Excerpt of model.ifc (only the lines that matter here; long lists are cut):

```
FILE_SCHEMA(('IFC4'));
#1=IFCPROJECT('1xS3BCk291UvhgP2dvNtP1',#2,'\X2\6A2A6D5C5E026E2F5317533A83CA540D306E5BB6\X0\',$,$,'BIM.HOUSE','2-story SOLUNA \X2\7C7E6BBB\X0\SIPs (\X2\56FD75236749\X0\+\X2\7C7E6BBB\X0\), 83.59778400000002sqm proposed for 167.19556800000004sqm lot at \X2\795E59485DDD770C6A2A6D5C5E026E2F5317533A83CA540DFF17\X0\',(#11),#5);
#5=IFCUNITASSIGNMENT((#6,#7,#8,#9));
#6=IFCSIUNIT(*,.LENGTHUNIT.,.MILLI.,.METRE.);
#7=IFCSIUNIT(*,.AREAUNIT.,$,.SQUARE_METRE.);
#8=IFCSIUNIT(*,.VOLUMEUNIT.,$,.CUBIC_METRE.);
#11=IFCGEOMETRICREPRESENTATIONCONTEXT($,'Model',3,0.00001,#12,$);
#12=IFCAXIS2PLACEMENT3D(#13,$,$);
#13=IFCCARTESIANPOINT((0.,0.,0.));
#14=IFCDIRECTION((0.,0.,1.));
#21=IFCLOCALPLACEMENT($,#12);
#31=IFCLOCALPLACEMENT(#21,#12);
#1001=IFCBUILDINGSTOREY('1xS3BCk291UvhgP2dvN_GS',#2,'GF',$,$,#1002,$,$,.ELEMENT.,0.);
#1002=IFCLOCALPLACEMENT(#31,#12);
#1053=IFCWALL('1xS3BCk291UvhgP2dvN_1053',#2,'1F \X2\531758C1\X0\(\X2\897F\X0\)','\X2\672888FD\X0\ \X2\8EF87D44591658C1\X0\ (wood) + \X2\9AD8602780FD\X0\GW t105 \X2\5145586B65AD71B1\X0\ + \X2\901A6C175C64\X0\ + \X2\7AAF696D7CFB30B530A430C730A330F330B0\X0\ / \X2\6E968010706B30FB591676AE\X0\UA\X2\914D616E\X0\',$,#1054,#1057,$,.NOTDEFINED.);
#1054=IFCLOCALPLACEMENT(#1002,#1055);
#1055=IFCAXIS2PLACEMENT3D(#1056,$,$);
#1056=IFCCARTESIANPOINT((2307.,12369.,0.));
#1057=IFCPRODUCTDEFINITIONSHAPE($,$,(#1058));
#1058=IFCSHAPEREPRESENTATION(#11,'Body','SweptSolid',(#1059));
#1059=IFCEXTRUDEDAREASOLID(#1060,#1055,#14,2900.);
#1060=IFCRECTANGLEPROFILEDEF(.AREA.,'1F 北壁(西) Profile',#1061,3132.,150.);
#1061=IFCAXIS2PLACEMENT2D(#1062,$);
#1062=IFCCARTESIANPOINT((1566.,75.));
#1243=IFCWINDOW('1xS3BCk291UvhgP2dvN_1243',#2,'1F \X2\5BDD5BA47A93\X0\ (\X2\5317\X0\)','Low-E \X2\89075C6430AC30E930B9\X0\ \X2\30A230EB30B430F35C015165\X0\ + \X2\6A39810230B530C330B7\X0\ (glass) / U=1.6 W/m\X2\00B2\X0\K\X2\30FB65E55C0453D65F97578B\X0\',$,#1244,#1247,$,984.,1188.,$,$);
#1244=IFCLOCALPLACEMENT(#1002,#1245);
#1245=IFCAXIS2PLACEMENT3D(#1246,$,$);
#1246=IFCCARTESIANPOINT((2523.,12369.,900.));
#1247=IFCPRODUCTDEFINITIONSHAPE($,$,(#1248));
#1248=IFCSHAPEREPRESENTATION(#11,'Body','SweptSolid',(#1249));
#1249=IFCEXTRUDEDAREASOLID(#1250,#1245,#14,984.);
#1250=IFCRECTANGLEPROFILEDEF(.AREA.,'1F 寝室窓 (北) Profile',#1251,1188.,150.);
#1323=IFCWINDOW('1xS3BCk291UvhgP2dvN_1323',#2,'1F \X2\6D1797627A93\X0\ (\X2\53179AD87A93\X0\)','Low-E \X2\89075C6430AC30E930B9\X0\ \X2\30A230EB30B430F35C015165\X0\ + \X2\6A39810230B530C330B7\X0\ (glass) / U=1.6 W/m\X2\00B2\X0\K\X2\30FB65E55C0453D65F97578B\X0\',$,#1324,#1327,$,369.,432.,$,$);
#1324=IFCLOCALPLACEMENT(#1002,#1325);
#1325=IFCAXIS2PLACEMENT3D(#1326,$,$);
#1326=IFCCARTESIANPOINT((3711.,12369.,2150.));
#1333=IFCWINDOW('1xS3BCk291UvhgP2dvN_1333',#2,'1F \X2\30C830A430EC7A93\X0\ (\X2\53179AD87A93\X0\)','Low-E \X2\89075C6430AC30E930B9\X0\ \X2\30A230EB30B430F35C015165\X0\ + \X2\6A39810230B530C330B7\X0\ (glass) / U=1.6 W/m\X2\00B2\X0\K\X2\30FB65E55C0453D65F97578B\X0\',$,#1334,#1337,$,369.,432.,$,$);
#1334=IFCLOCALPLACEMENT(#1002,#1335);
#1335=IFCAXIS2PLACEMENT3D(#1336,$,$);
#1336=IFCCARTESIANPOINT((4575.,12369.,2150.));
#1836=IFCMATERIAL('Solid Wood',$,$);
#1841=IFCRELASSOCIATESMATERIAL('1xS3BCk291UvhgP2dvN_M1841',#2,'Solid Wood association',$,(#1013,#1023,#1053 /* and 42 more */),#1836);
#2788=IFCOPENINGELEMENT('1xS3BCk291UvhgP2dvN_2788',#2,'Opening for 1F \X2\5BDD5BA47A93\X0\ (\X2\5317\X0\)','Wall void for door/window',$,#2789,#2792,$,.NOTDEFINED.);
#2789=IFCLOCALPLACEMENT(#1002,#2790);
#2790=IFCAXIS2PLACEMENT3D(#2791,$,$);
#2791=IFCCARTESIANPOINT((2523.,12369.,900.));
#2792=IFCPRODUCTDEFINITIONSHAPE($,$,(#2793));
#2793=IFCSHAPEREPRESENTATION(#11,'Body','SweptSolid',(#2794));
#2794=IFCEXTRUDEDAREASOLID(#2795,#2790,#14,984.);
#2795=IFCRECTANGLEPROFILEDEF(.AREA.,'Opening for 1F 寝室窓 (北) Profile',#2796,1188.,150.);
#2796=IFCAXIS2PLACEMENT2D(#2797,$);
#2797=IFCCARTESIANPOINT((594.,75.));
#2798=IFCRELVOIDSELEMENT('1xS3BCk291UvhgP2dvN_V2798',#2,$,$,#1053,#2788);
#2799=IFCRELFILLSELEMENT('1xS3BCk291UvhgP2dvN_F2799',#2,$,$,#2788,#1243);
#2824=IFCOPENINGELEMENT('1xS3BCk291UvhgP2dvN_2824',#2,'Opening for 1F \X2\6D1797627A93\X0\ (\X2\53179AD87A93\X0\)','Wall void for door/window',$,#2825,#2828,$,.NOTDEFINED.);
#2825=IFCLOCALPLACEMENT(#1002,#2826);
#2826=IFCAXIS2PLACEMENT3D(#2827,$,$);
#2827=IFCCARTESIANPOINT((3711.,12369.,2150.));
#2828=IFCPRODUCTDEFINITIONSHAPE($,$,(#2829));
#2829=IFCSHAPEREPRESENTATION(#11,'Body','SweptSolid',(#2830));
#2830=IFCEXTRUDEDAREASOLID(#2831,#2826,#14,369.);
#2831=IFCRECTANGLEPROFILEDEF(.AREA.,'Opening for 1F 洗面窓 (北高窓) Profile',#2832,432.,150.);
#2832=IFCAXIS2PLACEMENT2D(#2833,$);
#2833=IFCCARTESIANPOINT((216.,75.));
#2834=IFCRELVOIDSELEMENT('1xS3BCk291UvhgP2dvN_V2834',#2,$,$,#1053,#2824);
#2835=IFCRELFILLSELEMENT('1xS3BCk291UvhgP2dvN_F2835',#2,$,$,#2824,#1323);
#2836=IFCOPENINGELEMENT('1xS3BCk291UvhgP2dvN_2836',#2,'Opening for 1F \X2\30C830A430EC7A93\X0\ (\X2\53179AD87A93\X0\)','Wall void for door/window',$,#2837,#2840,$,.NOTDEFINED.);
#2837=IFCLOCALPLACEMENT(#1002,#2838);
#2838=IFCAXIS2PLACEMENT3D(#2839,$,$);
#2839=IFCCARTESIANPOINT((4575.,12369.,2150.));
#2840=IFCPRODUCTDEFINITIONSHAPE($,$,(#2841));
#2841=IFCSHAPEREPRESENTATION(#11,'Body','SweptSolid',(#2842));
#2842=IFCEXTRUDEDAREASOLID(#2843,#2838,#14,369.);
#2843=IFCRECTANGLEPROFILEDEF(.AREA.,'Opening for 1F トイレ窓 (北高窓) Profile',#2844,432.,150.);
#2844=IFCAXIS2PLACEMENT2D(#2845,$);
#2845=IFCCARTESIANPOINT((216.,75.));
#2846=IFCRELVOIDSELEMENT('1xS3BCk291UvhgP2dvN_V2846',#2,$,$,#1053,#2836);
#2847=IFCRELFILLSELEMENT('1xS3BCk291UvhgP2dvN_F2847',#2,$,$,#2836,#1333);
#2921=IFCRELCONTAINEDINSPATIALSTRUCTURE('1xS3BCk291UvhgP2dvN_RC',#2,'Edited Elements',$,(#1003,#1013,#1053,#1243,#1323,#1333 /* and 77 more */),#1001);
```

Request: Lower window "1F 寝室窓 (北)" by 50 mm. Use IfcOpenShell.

```python
import numpy as np
import ifcopenshell
import ifcopenshell.api.geometry
import ifcopenshell.util.placement
import ifcopenshell.util.unit

model = ifcopenshell.open("model.ifc")
unit_scale = ifcopenshell.util.unit.calculate_unit_scale(model)

window = model.by_guid("1xS3BCk291UvhgP2dvN_1243")
opening = window.FillsVoids[0].RelatingOpeningElement
dz = -0.05 / unit_scale

shift = np.array([0.0, 0.0, dz])
# The window is not placed relative to its opening, so move both.
for product in (opening, window):
    matrix = ifcopenshell.util.placement.get_local_placement(product.ObjectPlacement)
    matrix[:3, 3] += shift
    ifcopenshell.api.geometry.edit_object_placement(model, product=product, matrix=matrix, is_si=False)

print(f"moved by {dz * unit_scale:+.3f} m")

model.write("model_v2.ifc")
```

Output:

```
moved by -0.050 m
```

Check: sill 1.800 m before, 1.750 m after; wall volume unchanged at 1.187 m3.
